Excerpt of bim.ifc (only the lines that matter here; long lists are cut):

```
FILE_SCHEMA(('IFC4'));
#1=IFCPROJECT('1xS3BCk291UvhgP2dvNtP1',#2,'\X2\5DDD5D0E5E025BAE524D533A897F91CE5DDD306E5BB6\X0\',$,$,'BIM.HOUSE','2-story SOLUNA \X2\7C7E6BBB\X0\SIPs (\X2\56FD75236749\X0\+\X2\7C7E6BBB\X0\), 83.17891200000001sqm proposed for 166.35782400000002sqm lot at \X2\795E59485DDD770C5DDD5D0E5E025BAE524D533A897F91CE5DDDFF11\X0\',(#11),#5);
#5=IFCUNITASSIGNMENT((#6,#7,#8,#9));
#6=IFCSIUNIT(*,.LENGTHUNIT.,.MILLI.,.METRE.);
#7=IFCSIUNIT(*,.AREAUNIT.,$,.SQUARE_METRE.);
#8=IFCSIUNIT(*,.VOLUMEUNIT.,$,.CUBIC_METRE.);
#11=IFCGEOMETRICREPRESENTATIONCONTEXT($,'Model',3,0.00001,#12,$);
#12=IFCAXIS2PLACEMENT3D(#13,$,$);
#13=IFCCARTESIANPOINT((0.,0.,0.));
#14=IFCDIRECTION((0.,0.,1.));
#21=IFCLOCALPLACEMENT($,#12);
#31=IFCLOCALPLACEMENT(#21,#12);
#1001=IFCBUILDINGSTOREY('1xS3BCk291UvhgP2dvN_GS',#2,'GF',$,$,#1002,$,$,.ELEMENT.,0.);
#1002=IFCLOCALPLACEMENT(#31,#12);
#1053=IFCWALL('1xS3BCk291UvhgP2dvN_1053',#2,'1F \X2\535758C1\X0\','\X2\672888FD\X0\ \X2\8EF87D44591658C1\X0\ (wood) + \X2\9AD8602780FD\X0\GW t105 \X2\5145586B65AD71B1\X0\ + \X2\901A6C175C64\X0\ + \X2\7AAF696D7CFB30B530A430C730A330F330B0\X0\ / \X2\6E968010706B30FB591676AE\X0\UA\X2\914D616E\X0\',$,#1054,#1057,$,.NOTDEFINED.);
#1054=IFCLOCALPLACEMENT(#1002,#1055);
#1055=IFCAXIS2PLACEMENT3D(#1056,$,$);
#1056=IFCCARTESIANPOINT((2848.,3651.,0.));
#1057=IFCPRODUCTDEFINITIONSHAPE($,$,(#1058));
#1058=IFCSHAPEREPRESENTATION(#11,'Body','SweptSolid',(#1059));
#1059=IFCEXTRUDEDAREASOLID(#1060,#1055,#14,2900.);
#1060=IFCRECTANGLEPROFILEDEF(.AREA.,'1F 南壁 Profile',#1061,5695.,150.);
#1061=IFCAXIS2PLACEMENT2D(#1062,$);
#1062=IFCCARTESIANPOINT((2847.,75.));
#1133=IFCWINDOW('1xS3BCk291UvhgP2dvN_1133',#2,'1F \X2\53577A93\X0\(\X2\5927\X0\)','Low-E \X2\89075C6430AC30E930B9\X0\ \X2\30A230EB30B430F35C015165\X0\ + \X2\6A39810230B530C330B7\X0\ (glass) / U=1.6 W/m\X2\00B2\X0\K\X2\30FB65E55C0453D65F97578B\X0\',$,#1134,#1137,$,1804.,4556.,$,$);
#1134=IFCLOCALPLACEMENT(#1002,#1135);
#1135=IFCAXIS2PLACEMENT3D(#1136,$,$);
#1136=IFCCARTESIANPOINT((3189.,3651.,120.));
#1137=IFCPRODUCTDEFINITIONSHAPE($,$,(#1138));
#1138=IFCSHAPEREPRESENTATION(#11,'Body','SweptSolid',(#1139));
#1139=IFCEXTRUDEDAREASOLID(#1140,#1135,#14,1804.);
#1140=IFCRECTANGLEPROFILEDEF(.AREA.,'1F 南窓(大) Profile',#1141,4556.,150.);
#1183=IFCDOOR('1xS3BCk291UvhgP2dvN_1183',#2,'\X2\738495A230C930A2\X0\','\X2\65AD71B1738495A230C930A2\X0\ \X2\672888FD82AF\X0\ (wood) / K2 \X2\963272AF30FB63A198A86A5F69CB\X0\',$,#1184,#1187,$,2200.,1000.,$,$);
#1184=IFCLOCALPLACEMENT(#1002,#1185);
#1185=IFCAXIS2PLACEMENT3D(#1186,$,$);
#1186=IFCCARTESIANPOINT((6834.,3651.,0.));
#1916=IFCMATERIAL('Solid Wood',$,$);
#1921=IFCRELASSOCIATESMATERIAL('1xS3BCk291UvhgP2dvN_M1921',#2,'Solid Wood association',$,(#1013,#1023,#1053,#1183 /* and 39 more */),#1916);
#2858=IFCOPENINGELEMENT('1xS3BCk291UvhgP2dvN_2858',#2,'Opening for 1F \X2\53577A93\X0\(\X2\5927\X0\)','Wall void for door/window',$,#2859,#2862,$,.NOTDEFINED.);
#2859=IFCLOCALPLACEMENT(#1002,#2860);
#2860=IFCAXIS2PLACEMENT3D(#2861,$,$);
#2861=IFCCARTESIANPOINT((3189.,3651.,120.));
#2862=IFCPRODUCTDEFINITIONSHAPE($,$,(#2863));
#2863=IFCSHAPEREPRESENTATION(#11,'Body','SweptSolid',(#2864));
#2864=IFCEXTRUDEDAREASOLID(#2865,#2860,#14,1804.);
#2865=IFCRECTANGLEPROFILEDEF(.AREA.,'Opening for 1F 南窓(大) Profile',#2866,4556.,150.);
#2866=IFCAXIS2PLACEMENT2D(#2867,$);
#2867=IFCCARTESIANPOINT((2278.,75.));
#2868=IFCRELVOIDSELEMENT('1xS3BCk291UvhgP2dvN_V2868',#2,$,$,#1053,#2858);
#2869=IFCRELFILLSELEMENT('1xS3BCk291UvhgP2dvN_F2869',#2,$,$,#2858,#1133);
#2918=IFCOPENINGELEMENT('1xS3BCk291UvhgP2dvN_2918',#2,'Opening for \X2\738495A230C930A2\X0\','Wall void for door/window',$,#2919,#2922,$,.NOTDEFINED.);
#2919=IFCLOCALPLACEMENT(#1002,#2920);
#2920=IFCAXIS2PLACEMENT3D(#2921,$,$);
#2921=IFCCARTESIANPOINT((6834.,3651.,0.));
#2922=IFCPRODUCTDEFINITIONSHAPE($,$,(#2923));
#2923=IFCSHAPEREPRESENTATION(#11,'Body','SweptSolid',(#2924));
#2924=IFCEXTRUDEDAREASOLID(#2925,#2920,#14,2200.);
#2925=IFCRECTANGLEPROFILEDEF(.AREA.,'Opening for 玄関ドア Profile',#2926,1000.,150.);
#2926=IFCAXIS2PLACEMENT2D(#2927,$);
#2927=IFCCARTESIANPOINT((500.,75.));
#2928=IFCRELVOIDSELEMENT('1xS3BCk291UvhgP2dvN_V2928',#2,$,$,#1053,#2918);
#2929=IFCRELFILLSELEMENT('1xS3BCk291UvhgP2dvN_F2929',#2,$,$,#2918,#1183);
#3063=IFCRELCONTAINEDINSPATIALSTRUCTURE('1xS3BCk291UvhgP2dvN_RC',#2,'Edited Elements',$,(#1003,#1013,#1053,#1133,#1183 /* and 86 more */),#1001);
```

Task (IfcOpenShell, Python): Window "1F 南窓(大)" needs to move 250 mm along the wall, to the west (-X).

```python
import ifcopenshell
import ifcopenshell.api.geometry
import ifcopenshell.util.placement
import ifcopenshell.util.unit

model = ifcopenshell.open("bim.ifc")
unit_scale = ifcopenshell.util.unit.calculate_unit_scale(model)

window = model.by_guid("1xS3BCk291UvhgP2dvN_1133")
opening = window.FillsVoids[0].RelatingOpeningElement
wall = opening.VoidsElements[0].RelatingBuildingElement

wall_matrix = ifcopenshell.util.placement.get_local_placement(wall.ObjectPlacement)
shift = wall_matrix[:3, 0] * -0.25 / unit_scale
before = ifcopenshell.util.placement.get_local_placement(window.ObjectPlacement)[:3, 3].copy()

# The window is not placed relative to its opening, so move both.
for product in (opening, window):
    matrix = ifcopenshell.util.placement.get_local_placement(product.ObjectPlacement)
    matrix[:3, 3] += shift
    ifcopenshell.api.geometry.edit_object_placement(model, product=product, matrix=matrix, is_si=False)

after = ifcopenshell.util.placement.get_local_placement(window.ObjectPlacement)[:3, 3]
print("window moved by", (after - before).round(3) + 0.0)

model.write("bim_updated.ifc")
```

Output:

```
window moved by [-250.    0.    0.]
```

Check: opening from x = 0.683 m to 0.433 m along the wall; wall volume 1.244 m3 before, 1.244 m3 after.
